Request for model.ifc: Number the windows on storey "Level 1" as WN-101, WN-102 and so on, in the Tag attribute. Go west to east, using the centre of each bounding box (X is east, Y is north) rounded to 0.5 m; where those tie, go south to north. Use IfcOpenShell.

First a look at what the model holds.

```python
import ifcopenshell
import ifcopenshell.util.element
import ifcopenshell.util.placement

model = ifcopenshell.open("model.ifc")
print(model.schema)
storey = next(s for s in model.by_type("IfcBuildingStorey") if s.Name == "Level 1")
windows = [e for e in ifcopenshell.util.element.get_decomposition(storey) if e.is_a("IfcWindow")]
for e in sorted(windows, key=lambda e: e.id()):
    origin = ifcopenshell.util.placement.get_local_placement(e.ObjectPlacement)[:3, 3]
    print(e.id(), e.Tag, e.Name, origin.round(2) + 0.0, sep=" | ")
```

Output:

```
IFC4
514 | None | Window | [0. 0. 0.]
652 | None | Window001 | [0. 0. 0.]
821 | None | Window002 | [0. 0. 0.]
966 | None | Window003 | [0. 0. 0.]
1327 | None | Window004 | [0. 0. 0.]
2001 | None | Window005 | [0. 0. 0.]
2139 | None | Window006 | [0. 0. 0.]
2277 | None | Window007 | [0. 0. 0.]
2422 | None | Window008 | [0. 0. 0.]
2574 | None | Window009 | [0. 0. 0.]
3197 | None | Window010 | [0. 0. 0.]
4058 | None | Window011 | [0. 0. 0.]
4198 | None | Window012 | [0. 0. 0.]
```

```python
import ifcopenshell
import ifcopenshell.geom
import ifcopenshell.util.element
import ifcopenshell.util.shape

model = ifcopenshell.open("model.ifc")
settings = ifcopenshell.geom.settings()
settings.set("use-world-coords", True)


def centre(element):
    shape = ifcopenshell.geom.create_shape(settings, element)
    return ifcopenshell.util.shape.get_bbox_centroid(shape.geometry)


storey = next(s for s in model.by_type("IfcBuildingStorey") if s.Name == "Level 1")
windows = [e for e in ifcopenshell.util.element.get_decomposition(storey) if e.is_a("IfcWindow")]

# Insertion points can sit at a corner or the storey origin, so sort by the geometry (in metres).
centres = {e: centre(e) for e in windows}
windows.sort(key=lambda e: (round(centres[e][0] / 0.5), centres[e][1]))

for i, e in enumerate(windows, start=1):
    number = f"WN-1{i:02d}"
    e.Tag = number
    print(e.id(), number)

model.write("model_edited.ifc")
```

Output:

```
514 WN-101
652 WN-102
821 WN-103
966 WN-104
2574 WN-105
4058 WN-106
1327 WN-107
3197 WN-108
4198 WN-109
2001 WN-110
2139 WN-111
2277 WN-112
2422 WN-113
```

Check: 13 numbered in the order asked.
